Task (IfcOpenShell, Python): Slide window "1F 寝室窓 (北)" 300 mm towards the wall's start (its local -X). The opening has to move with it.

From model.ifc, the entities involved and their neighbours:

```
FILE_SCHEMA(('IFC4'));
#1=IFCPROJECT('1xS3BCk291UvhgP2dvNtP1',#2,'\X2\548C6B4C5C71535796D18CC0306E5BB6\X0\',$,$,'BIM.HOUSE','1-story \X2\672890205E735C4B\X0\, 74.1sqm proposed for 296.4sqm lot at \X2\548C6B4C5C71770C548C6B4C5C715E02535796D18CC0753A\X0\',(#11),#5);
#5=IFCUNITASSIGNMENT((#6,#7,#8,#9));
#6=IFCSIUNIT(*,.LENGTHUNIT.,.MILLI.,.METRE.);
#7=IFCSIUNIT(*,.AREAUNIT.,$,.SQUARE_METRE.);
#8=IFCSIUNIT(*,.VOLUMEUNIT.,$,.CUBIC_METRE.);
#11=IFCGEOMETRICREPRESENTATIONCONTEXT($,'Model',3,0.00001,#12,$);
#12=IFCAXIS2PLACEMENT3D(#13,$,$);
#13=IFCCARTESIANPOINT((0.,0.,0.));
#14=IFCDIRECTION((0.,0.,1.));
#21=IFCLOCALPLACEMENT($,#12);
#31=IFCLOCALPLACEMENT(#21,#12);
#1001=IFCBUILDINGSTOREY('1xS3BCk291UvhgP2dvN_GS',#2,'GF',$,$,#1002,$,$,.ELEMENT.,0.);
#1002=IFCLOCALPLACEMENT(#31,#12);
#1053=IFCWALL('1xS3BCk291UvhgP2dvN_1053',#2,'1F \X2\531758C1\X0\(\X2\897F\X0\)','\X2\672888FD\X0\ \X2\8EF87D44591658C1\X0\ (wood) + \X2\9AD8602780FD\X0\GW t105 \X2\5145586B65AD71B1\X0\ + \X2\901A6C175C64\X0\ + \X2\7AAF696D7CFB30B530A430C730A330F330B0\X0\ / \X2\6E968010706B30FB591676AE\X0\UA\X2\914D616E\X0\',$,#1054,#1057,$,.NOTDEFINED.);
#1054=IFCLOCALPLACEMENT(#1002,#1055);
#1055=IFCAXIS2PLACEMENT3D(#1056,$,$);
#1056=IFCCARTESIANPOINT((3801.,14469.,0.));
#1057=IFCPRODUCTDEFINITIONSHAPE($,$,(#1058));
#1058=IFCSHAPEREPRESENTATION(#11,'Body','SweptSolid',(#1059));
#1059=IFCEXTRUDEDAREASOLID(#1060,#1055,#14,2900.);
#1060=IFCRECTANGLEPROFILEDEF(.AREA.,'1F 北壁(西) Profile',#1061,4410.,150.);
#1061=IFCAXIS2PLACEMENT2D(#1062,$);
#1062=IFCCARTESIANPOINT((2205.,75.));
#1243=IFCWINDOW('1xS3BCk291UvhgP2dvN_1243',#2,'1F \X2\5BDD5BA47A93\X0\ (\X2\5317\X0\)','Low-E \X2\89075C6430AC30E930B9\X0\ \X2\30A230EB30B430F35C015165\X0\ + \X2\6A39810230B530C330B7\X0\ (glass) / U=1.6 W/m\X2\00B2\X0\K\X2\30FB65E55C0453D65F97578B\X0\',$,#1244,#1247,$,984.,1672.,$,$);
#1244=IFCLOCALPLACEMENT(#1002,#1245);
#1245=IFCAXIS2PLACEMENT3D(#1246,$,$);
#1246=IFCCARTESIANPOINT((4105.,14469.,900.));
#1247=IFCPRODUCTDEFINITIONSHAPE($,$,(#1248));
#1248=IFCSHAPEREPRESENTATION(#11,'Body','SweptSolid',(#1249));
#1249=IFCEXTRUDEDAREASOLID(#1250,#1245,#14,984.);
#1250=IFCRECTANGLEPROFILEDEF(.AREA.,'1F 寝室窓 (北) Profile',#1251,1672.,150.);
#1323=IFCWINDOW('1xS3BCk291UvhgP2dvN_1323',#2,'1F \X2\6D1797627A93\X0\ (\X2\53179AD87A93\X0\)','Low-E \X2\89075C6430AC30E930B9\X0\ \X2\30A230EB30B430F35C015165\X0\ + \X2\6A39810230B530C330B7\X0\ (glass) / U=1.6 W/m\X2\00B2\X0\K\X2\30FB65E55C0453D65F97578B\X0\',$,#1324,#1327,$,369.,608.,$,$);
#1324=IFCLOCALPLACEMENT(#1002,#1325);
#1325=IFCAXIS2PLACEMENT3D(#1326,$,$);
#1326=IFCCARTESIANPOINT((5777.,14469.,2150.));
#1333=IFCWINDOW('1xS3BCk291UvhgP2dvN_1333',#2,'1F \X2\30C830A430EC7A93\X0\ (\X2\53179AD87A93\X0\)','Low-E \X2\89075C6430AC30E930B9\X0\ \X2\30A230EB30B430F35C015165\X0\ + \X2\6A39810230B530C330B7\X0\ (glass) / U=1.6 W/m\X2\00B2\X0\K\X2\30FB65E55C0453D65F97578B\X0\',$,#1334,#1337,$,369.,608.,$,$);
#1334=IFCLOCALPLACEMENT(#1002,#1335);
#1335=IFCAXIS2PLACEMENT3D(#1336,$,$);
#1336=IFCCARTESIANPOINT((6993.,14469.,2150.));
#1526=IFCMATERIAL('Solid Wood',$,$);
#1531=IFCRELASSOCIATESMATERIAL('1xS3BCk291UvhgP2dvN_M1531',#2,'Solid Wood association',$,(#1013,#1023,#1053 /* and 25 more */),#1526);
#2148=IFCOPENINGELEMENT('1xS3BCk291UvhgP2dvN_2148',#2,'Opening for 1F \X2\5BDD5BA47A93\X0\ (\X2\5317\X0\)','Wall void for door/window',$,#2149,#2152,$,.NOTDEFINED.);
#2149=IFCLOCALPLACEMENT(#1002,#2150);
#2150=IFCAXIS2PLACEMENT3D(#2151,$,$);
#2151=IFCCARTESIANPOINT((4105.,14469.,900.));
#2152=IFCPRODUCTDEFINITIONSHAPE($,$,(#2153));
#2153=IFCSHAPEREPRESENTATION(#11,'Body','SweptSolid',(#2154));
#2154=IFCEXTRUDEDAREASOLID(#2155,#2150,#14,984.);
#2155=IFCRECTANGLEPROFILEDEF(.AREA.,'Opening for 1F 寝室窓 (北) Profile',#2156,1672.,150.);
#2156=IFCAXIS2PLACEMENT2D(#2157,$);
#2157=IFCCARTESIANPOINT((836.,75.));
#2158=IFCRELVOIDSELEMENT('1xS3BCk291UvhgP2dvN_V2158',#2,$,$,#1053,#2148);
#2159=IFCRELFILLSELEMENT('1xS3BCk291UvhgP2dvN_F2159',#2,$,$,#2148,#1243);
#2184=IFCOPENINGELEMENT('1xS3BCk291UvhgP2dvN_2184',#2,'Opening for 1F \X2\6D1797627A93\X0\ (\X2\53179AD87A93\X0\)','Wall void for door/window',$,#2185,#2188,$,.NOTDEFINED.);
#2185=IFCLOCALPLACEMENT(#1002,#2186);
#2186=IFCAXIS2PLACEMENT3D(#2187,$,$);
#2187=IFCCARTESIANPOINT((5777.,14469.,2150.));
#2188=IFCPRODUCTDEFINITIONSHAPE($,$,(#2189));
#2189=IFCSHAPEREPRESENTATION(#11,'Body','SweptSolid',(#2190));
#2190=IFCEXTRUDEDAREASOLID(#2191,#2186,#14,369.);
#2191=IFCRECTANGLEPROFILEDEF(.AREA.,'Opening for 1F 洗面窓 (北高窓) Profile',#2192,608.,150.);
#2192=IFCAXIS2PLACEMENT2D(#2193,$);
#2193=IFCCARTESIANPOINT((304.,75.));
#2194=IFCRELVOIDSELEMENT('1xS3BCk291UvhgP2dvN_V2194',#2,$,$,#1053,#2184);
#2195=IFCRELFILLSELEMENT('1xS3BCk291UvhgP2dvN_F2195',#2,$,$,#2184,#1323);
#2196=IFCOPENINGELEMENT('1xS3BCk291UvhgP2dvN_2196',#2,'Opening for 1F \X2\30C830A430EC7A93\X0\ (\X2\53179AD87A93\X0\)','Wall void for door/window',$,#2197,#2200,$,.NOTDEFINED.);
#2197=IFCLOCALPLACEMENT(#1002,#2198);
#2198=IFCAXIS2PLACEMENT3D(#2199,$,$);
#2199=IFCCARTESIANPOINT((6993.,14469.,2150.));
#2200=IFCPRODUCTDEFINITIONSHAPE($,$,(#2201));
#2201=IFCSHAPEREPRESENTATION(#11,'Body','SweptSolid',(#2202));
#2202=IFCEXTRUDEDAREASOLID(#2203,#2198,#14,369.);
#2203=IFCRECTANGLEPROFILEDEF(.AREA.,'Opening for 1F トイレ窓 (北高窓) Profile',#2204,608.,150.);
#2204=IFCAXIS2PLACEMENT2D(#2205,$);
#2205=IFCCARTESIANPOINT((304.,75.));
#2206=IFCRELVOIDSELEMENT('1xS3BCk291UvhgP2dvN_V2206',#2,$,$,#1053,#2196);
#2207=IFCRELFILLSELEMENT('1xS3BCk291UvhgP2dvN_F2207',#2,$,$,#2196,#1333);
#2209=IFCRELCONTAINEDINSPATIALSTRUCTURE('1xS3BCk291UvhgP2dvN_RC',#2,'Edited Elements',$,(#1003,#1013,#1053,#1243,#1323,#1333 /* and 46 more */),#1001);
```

```python
import ifcopenshell
import ifcopenshell.api.geometry
import ifcopenshell.util.placement
import ifcopenshell.util.unit

model = ifcopenshell.open("model.ifc")
unit_scale = ifcopenshell.util.unit.calculate_unit_scale(model)

window = model.by_guid("1xS3BCk291UvhgP2dvN_1243")
opening = window.FillsVoids[0].RelatingOpeningElement
wall = opening.VoidsElements[0].RelatingBuildingElement

wall_matrix = ifcopenshell.util.placement.get_local_placement(wall.ObjectPlacement)
shift = wall_matrix[:3, 0] * -0.3 / unit_scale
before = ifcopenshell.util.placement.get_local_placement(window.ObjectPlacement)[:3, 3].copy()

# The window is not placed relative to its opening, so move both.
for product in (opening, window):
    matrix = ifcopenshell.util.placement.get_local_placement(product.ObjectPlacement)
    matrix[:3, 3] += shift
    ifcopenshell.api.geometry.edit_object_placement(model, product=product, matrix=matrix, is_si=False)

after = ifcopenshell.util.placement.get_local_placement(window.ObjectPlacement)[:3, 3]
print("window moved by", (after - before).round(3) + 0.0)

model.write("model-out.ifc")
```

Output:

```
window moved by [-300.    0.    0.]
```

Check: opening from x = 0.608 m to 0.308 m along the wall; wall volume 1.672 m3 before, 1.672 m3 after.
